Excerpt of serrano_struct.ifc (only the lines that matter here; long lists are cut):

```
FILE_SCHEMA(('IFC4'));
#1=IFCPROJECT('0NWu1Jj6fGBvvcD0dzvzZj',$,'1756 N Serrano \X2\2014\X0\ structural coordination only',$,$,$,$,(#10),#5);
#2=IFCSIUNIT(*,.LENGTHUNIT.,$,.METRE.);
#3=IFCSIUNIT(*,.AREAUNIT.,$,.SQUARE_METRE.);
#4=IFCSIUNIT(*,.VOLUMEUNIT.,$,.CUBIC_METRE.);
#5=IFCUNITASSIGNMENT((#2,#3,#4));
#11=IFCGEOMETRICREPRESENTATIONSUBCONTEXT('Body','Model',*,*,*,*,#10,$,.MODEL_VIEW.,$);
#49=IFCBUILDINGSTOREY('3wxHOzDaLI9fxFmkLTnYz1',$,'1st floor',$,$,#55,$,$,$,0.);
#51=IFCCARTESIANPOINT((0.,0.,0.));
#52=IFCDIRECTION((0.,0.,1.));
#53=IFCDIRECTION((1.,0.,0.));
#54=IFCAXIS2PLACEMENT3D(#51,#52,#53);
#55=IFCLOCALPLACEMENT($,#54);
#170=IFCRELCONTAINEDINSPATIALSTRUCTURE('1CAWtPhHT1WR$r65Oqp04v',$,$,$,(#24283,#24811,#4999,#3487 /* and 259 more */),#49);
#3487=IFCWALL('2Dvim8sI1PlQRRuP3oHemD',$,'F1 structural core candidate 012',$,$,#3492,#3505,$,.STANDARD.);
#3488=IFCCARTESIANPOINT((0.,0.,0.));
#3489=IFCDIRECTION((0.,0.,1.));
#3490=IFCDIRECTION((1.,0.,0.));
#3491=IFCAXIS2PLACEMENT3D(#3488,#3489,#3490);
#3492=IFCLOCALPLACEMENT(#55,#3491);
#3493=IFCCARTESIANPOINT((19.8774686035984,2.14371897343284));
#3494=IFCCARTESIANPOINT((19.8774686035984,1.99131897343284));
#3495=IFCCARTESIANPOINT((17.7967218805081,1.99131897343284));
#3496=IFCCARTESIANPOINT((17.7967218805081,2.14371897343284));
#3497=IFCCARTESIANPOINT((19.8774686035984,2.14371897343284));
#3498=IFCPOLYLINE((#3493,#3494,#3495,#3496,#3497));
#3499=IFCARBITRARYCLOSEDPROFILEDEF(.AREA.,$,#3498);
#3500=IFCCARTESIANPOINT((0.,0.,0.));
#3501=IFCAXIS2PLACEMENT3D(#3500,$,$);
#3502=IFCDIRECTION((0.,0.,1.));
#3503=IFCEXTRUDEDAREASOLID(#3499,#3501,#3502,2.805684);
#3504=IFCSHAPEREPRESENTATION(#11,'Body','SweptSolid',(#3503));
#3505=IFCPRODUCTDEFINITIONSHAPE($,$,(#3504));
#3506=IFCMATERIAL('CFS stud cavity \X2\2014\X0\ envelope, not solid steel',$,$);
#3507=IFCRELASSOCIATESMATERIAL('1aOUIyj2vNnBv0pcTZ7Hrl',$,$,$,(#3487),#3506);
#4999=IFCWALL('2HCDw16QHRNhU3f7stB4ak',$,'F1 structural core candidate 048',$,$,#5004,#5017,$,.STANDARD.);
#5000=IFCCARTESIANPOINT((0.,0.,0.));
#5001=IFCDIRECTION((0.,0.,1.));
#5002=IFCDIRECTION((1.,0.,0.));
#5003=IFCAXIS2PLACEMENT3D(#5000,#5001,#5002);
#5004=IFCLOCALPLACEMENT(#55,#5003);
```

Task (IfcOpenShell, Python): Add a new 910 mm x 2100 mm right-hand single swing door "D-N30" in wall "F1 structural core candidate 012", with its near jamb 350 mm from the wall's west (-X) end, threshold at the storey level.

```python
import numpy as np
import ifcopenshell
import ifcopenshell.api.feature
import ifcopenshell.api.geometry
import ifcopenshell.api.root
import ifcopenshell.api.spatial
import ifcopenshell.geom
import ifcopenshell.util.element
import ifcopenshell.util.placement
import ifcopenshell.util.representation
import ifcopenshell.util.shape
import ifcopenshell.util.unit

model = ifcopenshell.open("serrano_struct.ifc")
unit_scale = ifcopenshell.util.unit.calculate_unit_scale(model)
settings = ifcopenshell.geom.settings()


def volume(element):
    """Net volume in cubic metres, openings subtracted."""
    shape = ifcopenshell.geom.create_shape(settings, element)
    return ifcopenshell.util.shape.get_volume(shape.geometry)


wall = model.by_id(3487)
storey = ifcopenshell.util.element.get_container(wall, ifc_class="IfcBuildingStorey")
context = ifcopenshell.util.representation.get_context(model, "Model", "Body", "MODEL_VIEW")
before = volume(wall)

width, height, from_end, sill = 0.91, 2.1, 0.35, 0.0  # metres

# The wall runs along its own X axis, and the end named is its -X end.
wall_shape = ifcopenshell.geom.create_shape(settings, wall)
x, y, z = ifcopenshell.util.shape.get_vertices(wall_shape.geometry).T
start = x.min() + from_end
face, thickness = float(y.min()), float(y.max() - y.min())
wall_matrix = ifcopenshell.util.placement.get_local_placement(wall.ObjectPlacement)
level = ifcopenshell.util.placement.get_local_placement(storey.ObjectPlacement)[2, 3]


def in_wall(x, y):
    """Placement at x, y metres in the wall's axes, at sill height."""
    matrix = wall_matrix.copy()
    matrix[:, 3] = wall_matrix @ np.array([x / unit_scale, y / unit_scale, 0.0, 1.0])
    matrix[2, 3] = level + sill / unit_scale
    return matrix


# Opening: a box that overshoots both wall faces by 50 mm.
opening = ifcopenshell.api.root.create_entity(model, ifc_class="IfcOpeningElement", predefined_type="OPENING")
box = ifcopenshell.api.geometry.add_wall_representation(
    model, context=context, length=width, height=height, thickness=thickness + 0.1
)
ifcopenshell.api.geometry.assign_representation(model, product=opening, representation=box)
ifcopenshell.api.geometry.edit_object_placement(model, product=opening, matrix=in_wall(start, face - 0.05), is_si=False)
ifcopenshell.api.feature.add_feature(model, feature=opening, element=wall)

door = ifcopenshell.api.root.create_entity(model, ifc_class="IfcDoor", name="D-N30", predefined_type="DOOR")
door.OverallWidth, door.OverallHeight = width / unit_scale, height / unit_scale
door.OperationType = "SINGLE_SWING_RIGHT"
body = ifcopenshell.api.geometry.add_door_representation(
    model,
    context=context,
    overall_width=door.OverallWidth,
    overall_height=door.OverallHeight,
    operation_type="SINGLE_SWING_RIGHT",
    lining_properties={"LiningDepth": thickness / unit_scale, "ThresholdDepth": thickness / unit_scale},
)
ifcopenshell.api.geometry.assign_representation(model, product=door, representation=body)
ifcopenshell.api.spatial.assign_container(model, products=[door], relating_structure=storey)
ifcopenshell.api.feature.add_filling(model, opening=opening, element=door)

# The lining spans the wall, so the door starts at the wall face.
ifcopenshell.api.geometry.edit_object_placement(model, product=door, matrix=in_wall(start, face), is_si=False)

after = volume(wall)

print(f"wall volume {before:.3f} -> {after:.3f} m3")

model.write("serrano_struct_v2.ifc")
```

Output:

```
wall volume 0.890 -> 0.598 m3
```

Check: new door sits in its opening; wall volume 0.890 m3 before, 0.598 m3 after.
